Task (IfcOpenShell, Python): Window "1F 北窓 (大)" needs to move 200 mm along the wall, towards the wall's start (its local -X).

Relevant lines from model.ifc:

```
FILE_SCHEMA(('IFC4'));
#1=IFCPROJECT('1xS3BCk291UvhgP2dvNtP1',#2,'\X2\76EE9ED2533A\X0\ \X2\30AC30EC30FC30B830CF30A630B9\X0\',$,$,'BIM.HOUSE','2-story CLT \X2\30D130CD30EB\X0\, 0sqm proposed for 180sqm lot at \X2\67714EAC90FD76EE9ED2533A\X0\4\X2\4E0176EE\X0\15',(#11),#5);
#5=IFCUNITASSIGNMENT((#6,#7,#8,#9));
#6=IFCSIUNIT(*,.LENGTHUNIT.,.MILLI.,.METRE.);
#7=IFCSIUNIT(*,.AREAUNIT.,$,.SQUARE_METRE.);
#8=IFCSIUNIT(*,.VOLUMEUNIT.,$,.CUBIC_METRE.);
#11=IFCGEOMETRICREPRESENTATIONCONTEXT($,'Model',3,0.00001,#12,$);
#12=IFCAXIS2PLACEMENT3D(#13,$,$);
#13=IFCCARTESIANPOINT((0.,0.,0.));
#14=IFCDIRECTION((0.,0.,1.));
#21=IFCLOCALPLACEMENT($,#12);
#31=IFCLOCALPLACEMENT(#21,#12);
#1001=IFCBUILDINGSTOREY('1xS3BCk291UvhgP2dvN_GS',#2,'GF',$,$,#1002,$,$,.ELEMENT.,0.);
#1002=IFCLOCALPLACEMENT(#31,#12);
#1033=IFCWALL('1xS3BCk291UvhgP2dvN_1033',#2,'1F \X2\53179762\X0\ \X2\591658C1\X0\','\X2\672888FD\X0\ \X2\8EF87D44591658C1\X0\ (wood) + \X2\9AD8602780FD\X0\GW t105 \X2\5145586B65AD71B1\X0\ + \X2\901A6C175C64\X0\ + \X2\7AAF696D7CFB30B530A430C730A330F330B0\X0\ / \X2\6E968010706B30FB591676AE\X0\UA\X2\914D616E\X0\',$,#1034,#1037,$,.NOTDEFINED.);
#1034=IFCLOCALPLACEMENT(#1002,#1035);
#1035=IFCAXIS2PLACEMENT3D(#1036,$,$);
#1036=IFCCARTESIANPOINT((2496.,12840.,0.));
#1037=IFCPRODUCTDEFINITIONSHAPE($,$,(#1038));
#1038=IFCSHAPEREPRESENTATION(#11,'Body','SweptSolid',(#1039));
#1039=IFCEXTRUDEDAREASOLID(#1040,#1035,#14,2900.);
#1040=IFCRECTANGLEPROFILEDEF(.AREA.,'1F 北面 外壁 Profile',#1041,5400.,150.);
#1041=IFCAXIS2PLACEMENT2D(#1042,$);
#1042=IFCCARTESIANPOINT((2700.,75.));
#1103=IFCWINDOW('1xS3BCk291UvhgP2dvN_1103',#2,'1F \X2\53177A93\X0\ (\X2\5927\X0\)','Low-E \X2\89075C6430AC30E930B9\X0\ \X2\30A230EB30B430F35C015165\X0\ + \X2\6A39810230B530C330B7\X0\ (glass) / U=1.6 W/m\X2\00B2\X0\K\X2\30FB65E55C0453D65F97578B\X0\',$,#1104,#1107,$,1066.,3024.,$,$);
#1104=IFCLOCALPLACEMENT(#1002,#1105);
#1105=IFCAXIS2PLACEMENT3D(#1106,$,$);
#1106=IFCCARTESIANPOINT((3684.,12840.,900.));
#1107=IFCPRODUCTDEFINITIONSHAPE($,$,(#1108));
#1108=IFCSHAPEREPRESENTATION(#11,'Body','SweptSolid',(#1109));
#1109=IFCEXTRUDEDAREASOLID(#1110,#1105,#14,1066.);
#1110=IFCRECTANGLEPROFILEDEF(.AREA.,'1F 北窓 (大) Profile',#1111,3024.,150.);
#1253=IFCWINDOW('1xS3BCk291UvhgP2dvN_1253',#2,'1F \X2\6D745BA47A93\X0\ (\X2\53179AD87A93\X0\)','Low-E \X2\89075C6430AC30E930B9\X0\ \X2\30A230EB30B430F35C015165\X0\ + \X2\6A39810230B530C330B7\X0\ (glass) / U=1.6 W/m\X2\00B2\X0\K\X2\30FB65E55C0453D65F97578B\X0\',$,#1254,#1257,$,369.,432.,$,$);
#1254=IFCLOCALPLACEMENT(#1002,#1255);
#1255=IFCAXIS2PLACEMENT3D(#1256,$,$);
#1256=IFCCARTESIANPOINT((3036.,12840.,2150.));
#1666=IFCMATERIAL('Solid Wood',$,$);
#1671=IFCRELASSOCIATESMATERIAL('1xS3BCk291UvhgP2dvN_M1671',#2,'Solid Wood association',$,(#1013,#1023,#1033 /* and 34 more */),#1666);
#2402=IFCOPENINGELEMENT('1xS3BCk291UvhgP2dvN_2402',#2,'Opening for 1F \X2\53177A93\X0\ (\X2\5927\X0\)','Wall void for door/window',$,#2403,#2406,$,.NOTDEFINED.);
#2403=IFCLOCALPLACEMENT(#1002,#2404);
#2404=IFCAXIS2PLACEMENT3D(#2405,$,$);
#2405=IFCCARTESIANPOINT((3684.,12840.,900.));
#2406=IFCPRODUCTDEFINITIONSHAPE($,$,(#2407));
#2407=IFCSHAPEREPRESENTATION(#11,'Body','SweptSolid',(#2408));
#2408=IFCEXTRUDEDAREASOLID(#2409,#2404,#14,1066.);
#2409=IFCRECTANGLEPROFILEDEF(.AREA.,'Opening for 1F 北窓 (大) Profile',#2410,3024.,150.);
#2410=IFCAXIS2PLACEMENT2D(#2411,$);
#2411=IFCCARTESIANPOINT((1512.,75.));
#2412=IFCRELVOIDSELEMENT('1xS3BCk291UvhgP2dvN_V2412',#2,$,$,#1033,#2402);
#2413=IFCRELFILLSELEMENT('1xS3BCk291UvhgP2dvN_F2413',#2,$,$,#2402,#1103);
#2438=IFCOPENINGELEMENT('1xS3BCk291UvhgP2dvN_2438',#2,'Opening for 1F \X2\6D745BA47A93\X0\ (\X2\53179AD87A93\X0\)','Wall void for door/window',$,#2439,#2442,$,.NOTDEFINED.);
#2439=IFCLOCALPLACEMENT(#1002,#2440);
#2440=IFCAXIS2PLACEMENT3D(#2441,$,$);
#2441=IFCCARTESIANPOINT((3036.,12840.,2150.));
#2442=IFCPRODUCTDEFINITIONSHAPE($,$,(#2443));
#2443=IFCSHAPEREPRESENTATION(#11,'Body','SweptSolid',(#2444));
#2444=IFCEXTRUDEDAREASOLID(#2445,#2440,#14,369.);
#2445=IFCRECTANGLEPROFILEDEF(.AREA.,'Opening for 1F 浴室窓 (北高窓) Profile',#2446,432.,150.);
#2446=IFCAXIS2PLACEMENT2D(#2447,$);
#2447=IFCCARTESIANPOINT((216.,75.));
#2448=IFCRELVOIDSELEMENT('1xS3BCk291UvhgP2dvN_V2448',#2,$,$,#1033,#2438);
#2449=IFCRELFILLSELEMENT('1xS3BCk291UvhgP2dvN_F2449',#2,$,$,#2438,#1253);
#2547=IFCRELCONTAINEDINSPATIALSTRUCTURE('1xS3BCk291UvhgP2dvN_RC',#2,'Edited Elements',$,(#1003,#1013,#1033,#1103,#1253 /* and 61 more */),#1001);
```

```python
import ifcopenshell
import ifcopenshell.api.geometry
import ifcopenshell.util.placement

model = ifcopenshell.open("model.ifc")

window = model.by_id(1103)
opening = window.FillsVoids[0].RelatingOpeningElement
wall = opening.VoidsElements[0].RelatingBuildingElement

wall_matrix = ifcopenshell.util.placement.get_local_placement(wall.ObjectPlacement)
shift = wall_matrix[:3, 0] * -200.0
before = ifcopenshell.util.placement.get_local_placement(window.ObjectPlacement)[:3, 3].copy()

# The window is not placed relative to its opening, so move both.
for product in (opening, window):
    matrix = ifcopenshell.util.placement.get_local_placement(product.ObjectPlacement)
    matrix[:3, 3] += shift
    ifcopenshell.api.geometry.edit_object_placement(model, product=product, matrix=matrix, is_si=False)

after = ifcopenshell.util.placement.get_local_placement(window.ObjectPlacement)[:3, 3]
print("window moved by", (after - before).round(3) + 0.0)

model.write("model_rev.ifc")
```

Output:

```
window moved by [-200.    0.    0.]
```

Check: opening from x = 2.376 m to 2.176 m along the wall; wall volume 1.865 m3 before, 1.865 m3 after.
